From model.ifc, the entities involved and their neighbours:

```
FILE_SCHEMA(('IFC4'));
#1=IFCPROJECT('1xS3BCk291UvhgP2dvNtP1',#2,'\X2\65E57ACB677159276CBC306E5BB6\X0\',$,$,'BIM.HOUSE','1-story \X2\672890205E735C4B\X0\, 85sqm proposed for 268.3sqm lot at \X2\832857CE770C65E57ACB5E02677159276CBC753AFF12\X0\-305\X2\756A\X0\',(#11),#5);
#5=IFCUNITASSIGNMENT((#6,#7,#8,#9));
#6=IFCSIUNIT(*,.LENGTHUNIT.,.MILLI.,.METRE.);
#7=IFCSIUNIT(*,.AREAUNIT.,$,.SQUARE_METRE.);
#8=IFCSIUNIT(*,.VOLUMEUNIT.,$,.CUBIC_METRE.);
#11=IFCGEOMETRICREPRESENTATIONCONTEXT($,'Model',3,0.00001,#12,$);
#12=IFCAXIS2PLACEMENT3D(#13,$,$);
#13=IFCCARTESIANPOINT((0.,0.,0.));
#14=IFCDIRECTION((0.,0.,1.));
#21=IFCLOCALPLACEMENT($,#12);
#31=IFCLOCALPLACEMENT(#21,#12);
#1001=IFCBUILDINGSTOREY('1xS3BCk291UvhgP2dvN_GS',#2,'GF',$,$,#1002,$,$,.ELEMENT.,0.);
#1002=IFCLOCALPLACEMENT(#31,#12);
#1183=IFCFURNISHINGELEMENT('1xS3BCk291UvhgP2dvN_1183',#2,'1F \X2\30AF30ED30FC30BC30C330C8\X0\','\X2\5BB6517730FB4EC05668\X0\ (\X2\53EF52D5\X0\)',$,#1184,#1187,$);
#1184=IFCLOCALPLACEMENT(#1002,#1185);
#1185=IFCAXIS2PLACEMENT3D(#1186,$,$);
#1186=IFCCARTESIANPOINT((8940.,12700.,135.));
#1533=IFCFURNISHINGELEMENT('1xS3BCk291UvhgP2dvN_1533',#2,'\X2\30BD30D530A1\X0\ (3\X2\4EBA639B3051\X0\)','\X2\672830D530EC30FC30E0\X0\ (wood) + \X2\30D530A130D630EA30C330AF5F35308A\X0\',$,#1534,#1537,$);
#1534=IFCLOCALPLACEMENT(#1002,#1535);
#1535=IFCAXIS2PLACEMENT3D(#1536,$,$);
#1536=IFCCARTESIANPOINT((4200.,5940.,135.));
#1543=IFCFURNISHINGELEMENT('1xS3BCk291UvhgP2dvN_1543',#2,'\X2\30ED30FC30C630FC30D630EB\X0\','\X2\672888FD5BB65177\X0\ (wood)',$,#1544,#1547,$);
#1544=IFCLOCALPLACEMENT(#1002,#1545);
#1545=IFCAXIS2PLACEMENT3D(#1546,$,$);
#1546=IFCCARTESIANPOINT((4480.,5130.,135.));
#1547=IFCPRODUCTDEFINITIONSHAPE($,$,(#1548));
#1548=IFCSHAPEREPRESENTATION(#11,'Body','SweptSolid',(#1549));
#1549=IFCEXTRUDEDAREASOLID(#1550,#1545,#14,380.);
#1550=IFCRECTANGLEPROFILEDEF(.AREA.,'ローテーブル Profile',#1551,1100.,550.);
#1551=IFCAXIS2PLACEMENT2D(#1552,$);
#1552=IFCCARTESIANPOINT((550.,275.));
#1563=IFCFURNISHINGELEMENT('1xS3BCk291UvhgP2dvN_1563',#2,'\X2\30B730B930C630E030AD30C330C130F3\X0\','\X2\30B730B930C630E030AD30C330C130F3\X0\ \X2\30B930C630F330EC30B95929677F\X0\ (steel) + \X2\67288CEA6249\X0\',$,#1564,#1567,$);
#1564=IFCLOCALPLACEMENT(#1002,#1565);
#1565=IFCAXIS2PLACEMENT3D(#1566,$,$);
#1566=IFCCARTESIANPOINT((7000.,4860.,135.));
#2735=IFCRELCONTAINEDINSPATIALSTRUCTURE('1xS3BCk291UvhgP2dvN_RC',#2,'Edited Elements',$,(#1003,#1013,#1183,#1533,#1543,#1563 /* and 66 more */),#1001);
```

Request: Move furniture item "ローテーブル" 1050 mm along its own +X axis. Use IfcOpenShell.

```python
import ifcopenshell
import ifcopenshell.api.geometry
import ifcopenshell.util.placement

model = ifcopenshell.open("model.ifc")

item = model.by_id(1543)
matrix = ifcopenshell.util.placement.get_local_placement(item.ObjectPlacement)
matrix[:3, 3] += matrix[:3, 0] * 1050.0
ifcopenshell.api.geometry.edit_object_placement(model, product=item, matrix=matrix, is_si=False)

print(ifcopenshell.util.placement.get_local_placement(item.ObjectPlacement).round(3) + 0.0)

model.write("model-out.ifc")
```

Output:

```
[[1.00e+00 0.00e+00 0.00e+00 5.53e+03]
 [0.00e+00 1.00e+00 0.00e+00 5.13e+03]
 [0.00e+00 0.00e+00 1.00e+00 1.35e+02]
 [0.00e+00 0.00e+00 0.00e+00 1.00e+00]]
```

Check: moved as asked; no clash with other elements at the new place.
